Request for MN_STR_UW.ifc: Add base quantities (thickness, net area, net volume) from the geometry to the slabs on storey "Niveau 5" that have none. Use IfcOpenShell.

First a look at what the model holds.

```python
import ifcopenshell
import ifcopenshell.util.element
import ifcopenshell.util.unit

model = ifcopenshell.open("MN_STR_UW.ifc")
print(model.schema)
for unit_type in ("LENGTHUNIT", "AREAUNIT", "VOLUMEUNIT"):
    print(unit_type, ifcopenshell.util.unit.calculate_unit_scale(model, unit_type))
storey = next(s for s in model.by_type("IfcBuildingStorey") if s.Name == "Niveau 5")
slabs = [e for e in ifcopenshell.util.element.get_decomposition(storey) if e.is_a("IfcSlab")]
for e in sorted(slabs, key=lambda e: e.id()):
    print(e.id(), e.is_a(), e.Name, list(ifcopenshell.util.element.get_psets(e, qtos_only=True)), sep=" | ")
```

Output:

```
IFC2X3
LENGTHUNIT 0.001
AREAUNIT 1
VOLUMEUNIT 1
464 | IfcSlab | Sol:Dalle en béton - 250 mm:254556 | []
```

```python
import ifcopenshell
import ifcopenshell.api.pset
import ifcopenshell.geom
import ifcopenshell.util.element
import ifcopenshell.util.shape
import ifcopenshell.util.unit

model = ifcopenshell.open("MN_STR_UW.ifc")
unit_scale = ifcopenshell.util.unit.calculate_unit_scale(model)
area_scale = ifcopenshell.util.unit.calculate_unit_scale(model, "AREAUNIT")
volume_scale = ifcopenshell.util.unit.calculate_unit_scale(model, "VOLUMEUNIT")
settings = ifcopenshell.geom.settings()

storey = next(s for s in model.by_type("IfcBuildingStorey") if s.Name == "Niveau 5")
slabs = [e for e in ifcopenshell.util.element.get_decomposition(storey) if e.is_a("IfcSlab")]

for e in sorted(slabs, key=lambda e: e.id()):
    if ifcopenshell.util.element.get_psets(e, qtos_only=True, should_inherit=False):
        continue
    # Geometry comes back in metres, in the element's own axes.
    shape = ifcopenshell.geom.create_shape(settings, e)
    values = {
        "Width": ifcopenshell.util.shape.get_z(shape.geometry) / unit_scale,
        "NetArea": ifcopenshell.util.shape.get_footprint_area(shape.geometry) / area_scale,
        "NetVolume": ifcopenshell.util.shape.get_volume(shape.geometry) / volume_scale,
    }
    qto = ifcopenshell.api.pset.add_qto(model, product=e, name="BaseQuantities")
    ifcopenshell.api.pset.edit_qto(model, qto=qto, properties=values)
    print(e.id(), {k: round(v, 3) for k, v in values.items()})

model.write("MN_STR_UW_rev.ifc")
```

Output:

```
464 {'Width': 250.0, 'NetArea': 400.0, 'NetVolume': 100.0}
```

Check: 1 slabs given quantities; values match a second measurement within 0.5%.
